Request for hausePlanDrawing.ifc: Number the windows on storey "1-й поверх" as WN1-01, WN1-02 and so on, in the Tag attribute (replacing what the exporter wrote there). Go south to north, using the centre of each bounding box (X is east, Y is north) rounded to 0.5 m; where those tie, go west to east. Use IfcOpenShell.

First a look at what the model holds.

```python
import ifcopenshell
import ifcopenshell.util.element
import ifcopenshell.util.placement

model = ifcopenshell.open("hausePlanDrawing.ifc")
print(model.schema)
storey = next(s for s in model.by_type("IfcBuildingStorey") if s.Name == "1-й поверх")
windows = [e for e in ifcopenshell.util.element.get_decomposition(storey) if e.is_a("IfcWindow")]
for e in sorted(windows, key=lambda e: e.id()):
    origin = ifcopenshell.util.placement.get_local_placement(e.ObjectPlacement)[:3, 3]
    print(e.id(), e.Tag, e.Name, origin.round(2) + 0.0, sep=" | ")
```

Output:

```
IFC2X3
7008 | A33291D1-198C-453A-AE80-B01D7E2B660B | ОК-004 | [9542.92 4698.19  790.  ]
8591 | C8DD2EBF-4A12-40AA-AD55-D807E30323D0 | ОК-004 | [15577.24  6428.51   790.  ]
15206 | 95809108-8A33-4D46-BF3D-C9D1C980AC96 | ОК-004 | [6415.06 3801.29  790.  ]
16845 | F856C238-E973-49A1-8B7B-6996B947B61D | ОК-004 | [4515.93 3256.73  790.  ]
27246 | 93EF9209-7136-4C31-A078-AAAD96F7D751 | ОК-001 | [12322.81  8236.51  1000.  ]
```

```python
import ifcopenshell
import ifcopenshell.geom
import ifcopenshell.util.element
import ifcopenshell.util.shape

model = ifcopenshell.open("hausePlanDrawing.ifc")
settings = ifcopenshell.geom.settings()
settings.set("use-world-coords", True)


def centre(element):
    shape = ifcopenshell.geom.create_shape(settings, element)
    return ifcopenshell.util.shape.get_bbox_centroid(shape.geometry)


storey = next(s for s in model.by_type("IfcBuildingStorey") if s.Name == "1-й поверх")
windows = [e for e in ifcopenshell.util.element.get_decomposition(storey) if e.is_a("IfcWindow")]

# Insertion points can sit at a corner or the storey origin, so sort by the geometry (in metres).
centres = {e: centre(e) for e in windows}
windows.sort(key=lambda e: (round(centres[e][1] / 0.5), centres[e][0]))

for i, e in enumerate(windows, start=1):
    number = f"WN1-{i:02d}"
    e.Tag = number
    print(e.id(), number)

model.write("hausePlanDrawing_edited.ifc")
```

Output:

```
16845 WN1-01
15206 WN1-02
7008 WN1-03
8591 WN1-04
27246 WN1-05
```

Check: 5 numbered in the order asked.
